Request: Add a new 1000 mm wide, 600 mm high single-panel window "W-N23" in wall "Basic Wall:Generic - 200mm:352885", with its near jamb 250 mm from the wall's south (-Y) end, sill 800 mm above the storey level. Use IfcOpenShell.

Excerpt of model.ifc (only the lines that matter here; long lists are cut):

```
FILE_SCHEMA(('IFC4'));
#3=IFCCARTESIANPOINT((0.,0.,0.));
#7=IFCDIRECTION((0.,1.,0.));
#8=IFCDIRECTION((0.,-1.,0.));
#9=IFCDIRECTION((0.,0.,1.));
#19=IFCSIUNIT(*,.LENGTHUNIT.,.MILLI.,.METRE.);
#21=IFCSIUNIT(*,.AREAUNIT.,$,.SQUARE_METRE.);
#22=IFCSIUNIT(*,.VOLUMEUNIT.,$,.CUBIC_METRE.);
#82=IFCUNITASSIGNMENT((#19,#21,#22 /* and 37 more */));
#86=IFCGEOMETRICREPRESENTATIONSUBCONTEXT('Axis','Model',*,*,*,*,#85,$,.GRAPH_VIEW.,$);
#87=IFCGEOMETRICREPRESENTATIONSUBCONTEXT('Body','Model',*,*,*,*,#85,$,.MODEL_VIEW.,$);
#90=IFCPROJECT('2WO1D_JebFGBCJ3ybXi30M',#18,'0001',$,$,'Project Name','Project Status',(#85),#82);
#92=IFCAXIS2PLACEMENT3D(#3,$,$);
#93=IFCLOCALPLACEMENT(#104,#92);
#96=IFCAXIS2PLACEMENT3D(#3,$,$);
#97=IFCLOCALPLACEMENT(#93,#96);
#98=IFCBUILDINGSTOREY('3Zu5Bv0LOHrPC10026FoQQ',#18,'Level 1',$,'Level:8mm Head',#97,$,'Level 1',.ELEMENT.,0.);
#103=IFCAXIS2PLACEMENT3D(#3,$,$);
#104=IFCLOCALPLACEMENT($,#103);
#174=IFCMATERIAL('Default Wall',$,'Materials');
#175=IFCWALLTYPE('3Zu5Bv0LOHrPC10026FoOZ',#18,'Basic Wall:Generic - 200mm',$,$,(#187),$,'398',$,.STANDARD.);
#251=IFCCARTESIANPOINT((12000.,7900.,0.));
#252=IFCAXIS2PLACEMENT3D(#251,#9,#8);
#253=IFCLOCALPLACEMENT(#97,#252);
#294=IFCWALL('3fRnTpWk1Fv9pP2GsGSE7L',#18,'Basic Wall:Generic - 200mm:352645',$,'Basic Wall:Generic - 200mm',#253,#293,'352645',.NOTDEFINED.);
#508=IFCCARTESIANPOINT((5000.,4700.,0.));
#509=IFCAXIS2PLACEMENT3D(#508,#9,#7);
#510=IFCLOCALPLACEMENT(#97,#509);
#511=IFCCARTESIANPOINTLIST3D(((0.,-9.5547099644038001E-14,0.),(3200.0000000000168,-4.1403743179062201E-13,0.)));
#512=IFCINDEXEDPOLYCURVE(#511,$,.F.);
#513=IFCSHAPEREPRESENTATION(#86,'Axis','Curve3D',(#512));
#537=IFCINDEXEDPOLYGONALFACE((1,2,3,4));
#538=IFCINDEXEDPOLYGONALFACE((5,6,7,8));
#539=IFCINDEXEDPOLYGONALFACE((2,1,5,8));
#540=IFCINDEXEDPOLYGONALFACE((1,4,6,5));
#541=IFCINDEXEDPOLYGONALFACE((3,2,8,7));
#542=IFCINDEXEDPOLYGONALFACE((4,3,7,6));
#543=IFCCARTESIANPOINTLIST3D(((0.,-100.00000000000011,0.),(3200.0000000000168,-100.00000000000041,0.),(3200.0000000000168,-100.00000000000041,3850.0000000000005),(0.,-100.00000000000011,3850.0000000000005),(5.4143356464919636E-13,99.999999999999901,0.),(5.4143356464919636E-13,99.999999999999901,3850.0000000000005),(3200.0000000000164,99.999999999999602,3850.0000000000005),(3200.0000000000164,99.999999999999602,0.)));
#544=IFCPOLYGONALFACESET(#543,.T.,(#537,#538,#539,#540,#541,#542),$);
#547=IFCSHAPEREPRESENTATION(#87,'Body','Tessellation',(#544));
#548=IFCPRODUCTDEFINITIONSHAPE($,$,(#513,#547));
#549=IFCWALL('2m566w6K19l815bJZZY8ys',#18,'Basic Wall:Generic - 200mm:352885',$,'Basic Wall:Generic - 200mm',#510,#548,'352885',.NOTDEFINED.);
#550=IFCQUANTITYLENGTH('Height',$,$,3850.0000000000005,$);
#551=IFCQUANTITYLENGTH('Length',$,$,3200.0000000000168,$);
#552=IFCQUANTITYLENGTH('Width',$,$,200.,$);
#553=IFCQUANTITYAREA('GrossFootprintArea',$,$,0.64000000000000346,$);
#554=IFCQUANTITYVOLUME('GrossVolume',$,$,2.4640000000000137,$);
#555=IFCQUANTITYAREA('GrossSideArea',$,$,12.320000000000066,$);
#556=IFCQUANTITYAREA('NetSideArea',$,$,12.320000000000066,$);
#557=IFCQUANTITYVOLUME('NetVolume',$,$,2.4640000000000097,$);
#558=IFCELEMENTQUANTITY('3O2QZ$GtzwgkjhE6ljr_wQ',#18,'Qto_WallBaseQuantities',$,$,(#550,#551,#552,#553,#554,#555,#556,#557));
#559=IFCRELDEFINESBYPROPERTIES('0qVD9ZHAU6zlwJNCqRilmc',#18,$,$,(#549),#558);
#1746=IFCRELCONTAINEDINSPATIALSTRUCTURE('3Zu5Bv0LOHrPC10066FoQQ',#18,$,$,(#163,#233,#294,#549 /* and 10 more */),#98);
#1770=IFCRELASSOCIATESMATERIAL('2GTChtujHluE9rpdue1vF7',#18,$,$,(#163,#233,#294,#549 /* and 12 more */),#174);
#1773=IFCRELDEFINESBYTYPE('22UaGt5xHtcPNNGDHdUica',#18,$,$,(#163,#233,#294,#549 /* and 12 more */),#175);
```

```python
import numpy as np
import ifcopenshell
import ifcopenshell.api.feature
import ifcopenshell.api.geometry
import ifcopenshell.api.pset
import ifcopenshell.api.root
import ifcopenshell.api.spatial
import ifcopenshell.geom
import ifcopenshell.util.element
import ifcopenshell.util.placement
import ifcopenshell.util.representation
import ifcopenshell.util.shape
import ifcopenshell.util.unit

model = ifcopenshell.open("model.ifc")
unit_scale = ifcopenshell.util.unit.calculate_unit_scale(model)
area_scale = ifcopenshell.util.unit.calculate_unit_scale(model, "AREAUNIT")
volume_scale = ifcopenshell.util.unit.calculate_unit_scale(model, "VOLUMEUNIT")
settings = ifcopenshell.geom.settings()


def volume(element):
    """Net volume in cubic metres, openings subtracted."""
    shape = ifcopenshell.geom.create_shape(settings, element)
    return ifcopenshell.util.shape.get_volume(shape.geometry)


wall = model.by_guid("2m566w6K19l815bJZZY8ys")
storey = ifcopenshell.util.element.get_container(wall, ifc_class="IfcBuildingStorey")
context = ifcopenshell.util.representation.get_context(model, "Model", "Body", "MODEL_VIEW")
before = volume(wall)

width, height, from_end, sill = 1, 0.6, 0.25, 0.8  # metres

# The wall runs along its own X axis, and the end named is its -X end.
wall_shape = ifcopenshell.geom.create_shape(settings, wall)
x, y, z = ifcopenshell.util.shape.get_vertices(wall_shape.geometry).T
start = x.min() + from_end
face, thickness = float(y.min()), float(y.max() - y.min())
wall_matrix = ifcopenshell.util.placement.get_local_placement(wall.ObjectPlacement)
level = ifcopenshell.util.placement.get_local_placement(storey.ObjectPlacement)[2, 3]


def in_wall(x, y):
    """Placement at x, y metres in the wall's axes, at sill height."""
    matrix = wall_matrix.copy()
    matrix[:, 3] = wall_matrix @ np.array([x / unit_scale, y / unit_scale, 0.0, 1.0])
    matrix[2, 3] = level + sill / unit_scale
    return matrix


# Opening: a box that overshoots both wall faces by 50 mm.
opening = ifcopenshell.api.root.create_entity(model, ifc_class="IfcOpeningElement", predefined_type="OPENING")
box = ifcopenshell.api.geometry.add_wall_representation(
    model, context=context, length=width, height=height, thickness=thickness + 0.1
)
ifcopenshell.api.geometry.assign_representation(model, product=opening, representation=box)
ifcopenshell.api.geometry.edit_object_placement(model, product=opening, matrix=in_wall(start, face - 0.05), is_si=False)
ifcopenshell.api.feature.add_feature(model, feature=opening, element=wall)

window = ifcopenshell.api.root.create_entity(model, ifc_class="IfcWindow", name="W-N23", predefined_type="WINDOW")
window.OverallWidth, window.OverallHeight = width / unit_scale, height / unit_scale
window.PartitioningType = "SINGLE_PANEL"
body = ifcopenshell.api.geometry.add_window_representation(
    model,
    context=context,
    overall_width=window.OverallWidth,
    overall_height=window.OverallHeight,
    partition_type="SINGLE_PANEL",
)
ifcopenshell.api.geometry.assign_representation(model, product=window, representation=body)
ifcopenshell.api.spatial.assign_container(model, products=[window], relating_structure=storey)
ifcopenshell.api.feature.add_filling(model, opening=opening, element=window)

# Centre the window in the wall's thickness.
ifcopenshell.api.geometry.edit_object_placement(model, product=window, matrix=in_wall(start, face), is_si=False)
window_shape = ifcopenshell.geom.create_shape(settings, window)
depth = ifcopenshell.util.shape.get_vertices(window_shape.geometry)[:, 1]
offset = face + thickness / 2 - (depth.min() + depth.max()) / 2
ifcopenshell.api.geometry.edit_object_placement(model, product=window, matrix=in_wall(start, offset), is_si=False)

after = volume(wall)

# Update the wall's stored quantities.
qto = model.by_id(ifcopenshell.util.element.get_pset(wall, "Qto_WallBaseQuantities", should_inherit=False)["id"])
ifcopenshell.api.pset.edit_qto(model, qto=qto, properties={
    "NetSideArea": after / thickness / area_scale,
    "NetVolume": after / volume_scale,
})

print(f"wall volume {before:.3f} -> {after:.3f} m3")

model.write("model_v2.ifc")
```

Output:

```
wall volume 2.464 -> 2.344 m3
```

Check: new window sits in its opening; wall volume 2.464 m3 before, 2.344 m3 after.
